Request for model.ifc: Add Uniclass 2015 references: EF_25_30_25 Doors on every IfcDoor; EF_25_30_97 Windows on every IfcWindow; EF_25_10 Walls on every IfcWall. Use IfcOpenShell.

First a look at what the model holds.

```python
import ifcopenshell

model = ifcopenshell.open("model.ifc")
print(model.schema)
print("classifications:", [c.Name for c in model.by_type("IfcClassification")])
for ifc_class in ("IfcDoor", "IfcRoof", "IfcStair", "IfcWall", "IfcWindow"):
    print(ifc_class, len(model.by_type(ifc_class)))
```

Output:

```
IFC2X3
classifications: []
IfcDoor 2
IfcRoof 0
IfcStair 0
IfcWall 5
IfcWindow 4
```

```python
import ifcopenshell
import ifcopenshell.api.classification

model = ifcopenshell.open("model.ifc")

# IFC2X3 requires Source and Edition and has no link from the project to the system.
system = model.create_entity("IfcClassification", Source="NBS", Edition="2015", Name="Uniclass 2015")

codes = {
    "IfcDoor": ("EF_25_30_25", "Doors"),
    "IfcWindow": ("EF_25_30_97", "Windows"),
    "IfcWall": ("EF_25_10", "Walls"),
}
for ifc_class, (code, name) in codes.items():
    products = model.by_type(ifc_class)
    ifcopenshell.api.classification.add_reference(
        model, products=products, classification=system, identification=code, name=name
    )
    print(code, len(products))

model.write("model_updated.ifc")
```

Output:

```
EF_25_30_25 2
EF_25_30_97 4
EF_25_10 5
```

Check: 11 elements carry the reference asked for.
